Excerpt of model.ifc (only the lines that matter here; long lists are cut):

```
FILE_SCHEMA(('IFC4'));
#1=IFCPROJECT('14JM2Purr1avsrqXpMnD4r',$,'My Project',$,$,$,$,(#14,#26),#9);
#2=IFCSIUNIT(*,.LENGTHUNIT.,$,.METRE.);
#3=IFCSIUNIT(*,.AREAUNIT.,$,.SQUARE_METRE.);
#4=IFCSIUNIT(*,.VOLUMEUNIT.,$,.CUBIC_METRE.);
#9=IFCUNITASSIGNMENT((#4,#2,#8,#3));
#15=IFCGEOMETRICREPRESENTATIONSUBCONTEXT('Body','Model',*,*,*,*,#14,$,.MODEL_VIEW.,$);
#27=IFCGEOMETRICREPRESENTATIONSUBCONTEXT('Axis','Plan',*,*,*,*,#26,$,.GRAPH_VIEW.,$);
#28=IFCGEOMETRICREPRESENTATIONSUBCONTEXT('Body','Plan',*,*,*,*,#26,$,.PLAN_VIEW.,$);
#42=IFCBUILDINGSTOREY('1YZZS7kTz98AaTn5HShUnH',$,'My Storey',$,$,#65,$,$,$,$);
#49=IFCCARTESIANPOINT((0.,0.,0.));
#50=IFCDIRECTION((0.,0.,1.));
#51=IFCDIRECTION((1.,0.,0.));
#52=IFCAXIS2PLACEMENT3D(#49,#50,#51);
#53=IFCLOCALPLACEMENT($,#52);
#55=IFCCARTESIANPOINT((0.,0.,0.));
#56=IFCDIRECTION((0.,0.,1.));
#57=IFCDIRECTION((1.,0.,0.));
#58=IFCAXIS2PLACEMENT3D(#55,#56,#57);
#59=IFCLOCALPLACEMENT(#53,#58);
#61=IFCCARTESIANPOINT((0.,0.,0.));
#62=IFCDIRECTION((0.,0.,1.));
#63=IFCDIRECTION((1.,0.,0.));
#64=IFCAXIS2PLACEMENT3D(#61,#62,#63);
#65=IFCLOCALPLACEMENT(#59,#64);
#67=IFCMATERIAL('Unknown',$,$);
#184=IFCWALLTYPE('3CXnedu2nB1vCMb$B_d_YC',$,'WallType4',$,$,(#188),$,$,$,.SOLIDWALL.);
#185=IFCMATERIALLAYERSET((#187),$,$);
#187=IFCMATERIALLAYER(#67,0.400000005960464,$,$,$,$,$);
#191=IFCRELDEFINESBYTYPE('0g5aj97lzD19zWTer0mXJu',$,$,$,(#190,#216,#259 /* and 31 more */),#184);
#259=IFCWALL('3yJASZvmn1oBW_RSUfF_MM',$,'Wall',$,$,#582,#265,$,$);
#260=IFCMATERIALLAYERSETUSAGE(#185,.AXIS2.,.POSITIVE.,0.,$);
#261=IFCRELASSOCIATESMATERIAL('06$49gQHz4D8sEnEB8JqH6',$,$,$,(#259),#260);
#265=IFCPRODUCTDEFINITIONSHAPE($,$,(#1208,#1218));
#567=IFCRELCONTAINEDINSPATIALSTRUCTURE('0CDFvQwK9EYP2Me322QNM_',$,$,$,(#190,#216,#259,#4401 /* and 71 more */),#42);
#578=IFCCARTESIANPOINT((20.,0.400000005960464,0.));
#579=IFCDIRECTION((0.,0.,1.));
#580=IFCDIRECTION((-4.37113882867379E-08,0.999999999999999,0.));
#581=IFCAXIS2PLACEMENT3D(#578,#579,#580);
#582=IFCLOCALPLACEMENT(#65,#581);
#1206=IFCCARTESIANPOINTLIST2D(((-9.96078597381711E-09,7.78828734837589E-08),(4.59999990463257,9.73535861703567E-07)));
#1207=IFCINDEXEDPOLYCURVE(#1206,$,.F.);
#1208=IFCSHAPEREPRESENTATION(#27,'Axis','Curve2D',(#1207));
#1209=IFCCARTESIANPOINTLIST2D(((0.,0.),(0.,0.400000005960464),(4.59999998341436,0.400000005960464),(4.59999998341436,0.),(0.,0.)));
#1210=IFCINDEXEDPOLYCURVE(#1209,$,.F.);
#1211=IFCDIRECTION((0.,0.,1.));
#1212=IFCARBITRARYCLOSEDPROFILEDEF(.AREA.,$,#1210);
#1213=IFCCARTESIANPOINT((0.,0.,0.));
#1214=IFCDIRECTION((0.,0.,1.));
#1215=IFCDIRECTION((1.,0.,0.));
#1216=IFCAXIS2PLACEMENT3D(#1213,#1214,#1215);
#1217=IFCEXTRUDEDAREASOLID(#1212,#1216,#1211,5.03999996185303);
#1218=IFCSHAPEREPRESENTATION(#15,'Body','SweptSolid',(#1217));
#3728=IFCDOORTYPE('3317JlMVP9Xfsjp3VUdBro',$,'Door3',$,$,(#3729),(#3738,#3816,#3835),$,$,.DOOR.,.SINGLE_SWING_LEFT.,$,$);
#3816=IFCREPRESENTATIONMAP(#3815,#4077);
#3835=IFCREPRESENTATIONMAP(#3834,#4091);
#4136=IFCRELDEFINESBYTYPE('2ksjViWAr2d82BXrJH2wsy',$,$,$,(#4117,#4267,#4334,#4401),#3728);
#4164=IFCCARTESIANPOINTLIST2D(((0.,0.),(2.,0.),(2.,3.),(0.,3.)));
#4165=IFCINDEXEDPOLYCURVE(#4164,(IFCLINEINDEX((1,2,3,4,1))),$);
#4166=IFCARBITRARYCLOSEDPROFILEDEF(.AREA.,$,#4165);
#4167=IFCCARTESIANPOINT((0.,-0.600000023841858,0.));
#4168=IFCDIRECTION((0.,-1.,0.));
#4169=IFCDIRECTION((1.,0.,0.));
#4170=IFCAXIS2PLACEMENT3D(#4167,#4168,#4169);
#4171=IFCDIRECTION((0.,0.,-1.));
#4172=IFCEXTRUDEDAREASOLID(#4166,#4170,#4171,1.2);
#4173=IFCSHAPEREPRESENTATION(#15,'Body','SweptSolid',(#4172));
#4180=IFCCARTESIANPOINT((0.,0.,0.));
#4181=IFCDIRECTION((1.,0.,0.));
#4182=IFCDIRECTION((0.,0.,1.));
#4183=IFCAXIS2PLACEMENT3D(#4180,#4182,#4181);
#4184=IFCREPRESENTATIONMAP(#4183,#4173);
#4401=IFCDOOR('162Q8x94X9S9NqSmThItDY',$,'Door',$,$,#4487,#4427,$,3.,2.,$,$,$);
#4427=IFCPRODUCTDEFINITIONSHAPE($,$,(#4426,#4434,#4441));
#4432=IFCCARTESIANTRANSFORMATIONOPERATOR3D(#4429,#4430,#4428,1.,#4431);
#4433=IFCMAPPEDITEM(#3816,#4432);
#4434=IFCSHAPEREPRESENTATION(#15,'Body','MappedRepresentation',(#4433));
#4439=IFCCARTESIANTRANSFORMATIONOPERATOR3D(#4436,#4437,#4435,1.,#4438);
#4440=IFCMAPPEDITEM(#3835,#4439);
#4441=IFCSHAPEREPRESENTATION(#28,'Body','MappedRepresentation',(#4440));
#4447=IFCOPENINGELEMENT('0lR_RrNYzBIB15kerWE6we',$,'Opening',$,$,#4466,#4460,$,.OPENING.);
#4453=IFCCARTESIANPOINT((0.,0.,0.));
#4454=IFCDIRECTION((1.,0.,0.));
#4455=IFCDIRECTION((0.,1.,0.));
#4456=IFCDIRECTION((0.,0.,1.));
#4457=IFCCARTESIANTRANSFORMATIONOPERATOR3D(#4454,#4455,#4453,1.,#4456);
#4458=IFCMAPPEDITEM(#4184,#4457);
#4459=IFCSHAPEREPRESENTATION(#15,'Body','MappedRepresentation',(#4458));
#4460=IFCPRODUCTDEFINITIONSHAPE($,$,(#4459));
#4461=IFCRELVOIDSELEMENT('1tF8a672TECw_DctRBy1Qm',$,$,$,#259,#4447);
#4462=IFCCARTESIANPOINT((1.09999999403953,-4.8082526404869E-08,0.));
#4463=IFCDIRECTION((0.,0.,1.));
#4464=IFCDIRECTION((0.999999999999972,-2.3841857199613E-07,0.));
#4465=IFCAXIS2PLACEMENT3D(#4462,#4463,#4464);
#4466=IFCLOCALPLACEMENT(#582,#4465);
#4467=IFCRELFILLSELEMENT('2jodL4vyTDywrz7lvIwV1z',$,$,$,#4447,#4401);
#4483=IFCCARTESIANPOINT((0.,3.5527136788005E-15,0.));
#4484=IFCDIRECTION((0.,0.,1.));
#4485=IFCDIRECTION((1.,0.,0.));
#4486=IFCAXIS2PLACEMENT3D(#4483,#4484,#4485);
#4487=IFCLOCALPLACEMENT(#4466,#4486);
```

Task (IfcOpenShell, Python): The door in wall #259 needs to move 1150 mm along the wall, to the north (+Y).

```python
import ifcopenshell
import ifcopenshell.api.geometry
import ifcopenshell.util.placement

model = ifcopenshell.open("model.ifc")

door = model.by_guid("162Q8x94X9S9NqSmThItDY")
opening = door.FillsVoids[0].RelatingOpeningElement
wall = opening.VoidsElements[0].RelatingBuildingElement

wall_matrix = ifcopenshell.util.placement.get_local_placement(wall.ObjectPlacement)
shift = wall_matrix[:3, 0] * 1.15
before = ifcopenshell.util.placement.get_local_placement(door.ObjectPlacement)[:3, 3].copy()

# The door is placed relative to its opening, so it follows when the opening moves.
matrix = ifcopenshell.util.placement.get_local_placement(opening.ObjectPlacement)
matrix[:3, 3] += shift
ifcopenshell.api.geometry.edit_object_placement(
    model, product=opening, matrix=matrix, is_si=False, should_transform_children=True
)

after = ifcopenshell.util.placement.get_local_placement(door.ObjectPlacement)[:3, 3]
print("door moved by", (after - before).round(3) + 0.0)

model.write("model-out.ifc")
```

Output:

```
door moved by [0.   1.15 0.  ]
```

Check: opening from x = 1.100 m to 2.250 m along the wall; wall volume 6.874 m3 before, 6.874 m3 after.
